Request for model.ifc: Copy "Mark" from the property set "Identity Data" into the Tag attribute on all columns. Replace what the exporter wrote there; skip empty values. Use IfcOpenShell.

First a look at what the model holds.

```python
import ifcopenshell
import ifcopenshell.util.element

model = ifcopenshell.open("model.ifc")
print(model.schema)
columns = model.by_type("IfcColumn")
print(len(columns), "columns")
for e in columns[:8]:
    source = ifcopenshell.util.element.get_pset(e, "Identity Data", "Mark")
    target = e.Tag
    print(e.id(), repr(source), repr(target), sep=" | ")
```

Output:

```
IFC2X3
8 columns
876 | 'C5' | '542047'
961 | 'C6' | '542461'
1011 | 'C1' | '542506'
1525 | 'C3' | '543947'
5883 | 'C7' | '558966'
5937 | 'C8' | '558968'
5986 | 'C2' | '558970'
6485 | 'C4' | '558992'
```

```python
import ifcopenshell
import ifcopenshell.util.element

model = ifcopenshell.open("model.ifc")

count = 0
for e in model.by_type("IfcColumn"):
    value = ifcopenshell.util.element.get_pset(e, "Identity Data", "Mark")
    current = e.Tag
    if not value or not value.strip() or current == value:
        continue
    e.Tag = value
    count += 1

print(count, "columns updated")

model.write("model_updated.ifc")
```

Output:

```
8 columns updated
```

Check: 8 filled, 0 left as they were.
